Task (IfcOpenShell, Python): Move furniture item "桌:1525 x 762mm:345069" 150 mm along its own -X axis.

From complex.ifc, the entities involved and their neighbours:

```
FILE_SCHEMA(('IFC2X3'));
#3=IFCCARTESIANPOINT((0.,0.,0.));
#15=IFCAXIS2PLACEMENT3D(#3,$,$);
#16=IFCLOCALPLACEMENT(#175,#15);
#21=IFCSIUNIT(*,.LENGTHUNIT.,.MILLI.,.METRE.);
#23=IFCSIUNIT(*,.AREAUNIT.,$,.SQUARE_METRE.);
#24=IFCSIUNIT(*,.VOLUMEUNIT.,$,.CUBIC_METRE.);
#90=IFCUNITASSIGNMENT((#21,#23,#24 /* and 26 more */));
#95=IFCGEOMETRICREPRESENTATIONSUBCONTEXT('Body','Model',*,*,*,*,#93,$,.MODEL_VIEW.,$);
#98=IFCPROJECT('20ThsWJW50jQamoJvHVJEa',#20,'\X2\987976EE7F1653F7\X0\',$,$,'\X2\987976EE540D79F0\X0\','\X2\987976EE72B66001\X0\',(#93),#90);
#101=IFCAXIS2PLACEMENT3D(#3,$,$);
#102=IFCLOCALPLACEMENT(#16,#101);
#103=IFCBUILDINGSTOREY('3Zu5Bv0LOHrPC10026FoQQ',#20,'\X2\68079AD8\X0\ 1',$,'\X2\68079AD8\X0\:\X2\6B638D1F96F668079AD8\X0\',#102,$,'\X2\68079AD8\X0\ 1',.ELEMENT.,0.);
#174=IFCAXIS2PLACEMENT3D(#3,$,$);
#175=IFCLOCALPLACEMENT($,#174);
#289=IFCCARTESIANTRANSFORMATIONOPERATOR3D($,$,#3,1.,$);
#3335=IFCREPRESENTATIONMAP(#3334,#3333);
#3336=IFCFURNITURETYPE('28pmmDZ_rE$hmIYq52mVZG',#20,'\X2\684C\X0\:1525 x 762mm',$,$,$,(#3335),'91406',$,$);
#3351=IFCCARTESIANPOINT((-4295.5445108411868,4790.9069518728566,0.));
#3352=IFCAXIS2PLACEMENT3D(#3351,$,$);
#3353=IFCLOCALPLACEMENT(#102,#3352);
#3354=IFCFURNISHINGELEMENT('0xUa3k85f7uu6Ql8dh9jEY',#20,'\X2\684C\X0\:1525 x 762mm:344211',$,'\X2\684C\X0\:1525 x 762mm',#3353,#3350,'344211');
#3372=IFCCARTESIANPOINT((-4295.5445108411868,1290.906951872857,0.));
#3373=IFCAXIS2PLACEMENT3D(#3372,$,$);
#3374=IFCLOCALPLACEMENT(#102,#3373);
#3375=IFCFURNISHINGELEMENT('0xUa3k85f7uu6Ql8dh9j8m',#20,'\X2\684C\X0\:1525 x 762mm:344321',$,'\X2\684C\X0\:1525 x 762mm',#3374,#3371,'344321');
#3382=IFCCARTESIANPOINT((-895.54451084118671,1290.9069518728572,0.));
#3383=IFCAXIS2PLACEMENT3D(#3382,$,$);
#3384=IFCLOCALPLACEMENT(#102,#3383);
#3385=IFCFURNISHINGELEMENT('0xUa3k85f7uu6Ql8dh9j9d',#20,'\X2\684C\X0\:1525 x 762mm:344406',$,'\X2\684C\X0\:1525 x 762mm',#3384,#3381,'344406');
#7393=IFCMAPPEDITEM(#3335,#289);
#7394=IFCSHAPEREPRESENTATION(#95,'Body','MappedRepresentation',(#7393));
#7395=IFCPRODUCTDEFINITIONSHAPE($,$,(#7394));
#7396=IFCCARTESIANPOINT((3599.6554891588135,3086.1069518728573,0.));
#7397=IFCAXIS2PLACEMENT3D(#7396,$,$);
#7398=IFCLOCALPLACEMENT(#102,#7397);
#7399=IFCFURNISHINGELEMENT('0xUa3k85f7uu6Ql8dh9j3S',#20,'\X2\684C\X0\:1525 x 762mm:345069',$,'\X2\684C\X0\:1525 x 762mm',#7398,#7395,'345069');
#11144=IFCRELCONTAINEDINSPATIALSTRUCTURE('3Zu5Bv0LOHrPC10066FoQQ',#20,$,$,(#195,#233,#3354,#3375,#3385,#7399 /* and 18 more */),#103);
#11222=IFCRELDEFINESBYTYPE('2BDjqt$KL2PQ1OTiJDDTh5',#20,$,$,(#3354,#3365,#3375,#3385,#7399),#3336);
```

```python
import ifcopenshell
import ifcopenshell.api.geometry
import ifcopenshell.util.placement

model = ifcopenshell.open("complex.ifc")

item = model.by_guid("0xUa3k85f7uu6Ql8dh9j3S")
matrix = ifcopenshell.util.placement.get_local_placement(item.ObjectPlacement)
matrix[:3, 3] -= matrix[:3, 0] * 150.0
ifcopenshell.api.geometry.edit_object_placement(model, product=item, matrix=matrix, is_si=False)

print(ifcopenshell.util.placement.get_local_placement(item.ObjectPlacement).round(3) + 0.0)

model.write("complex_rev.ifc")
```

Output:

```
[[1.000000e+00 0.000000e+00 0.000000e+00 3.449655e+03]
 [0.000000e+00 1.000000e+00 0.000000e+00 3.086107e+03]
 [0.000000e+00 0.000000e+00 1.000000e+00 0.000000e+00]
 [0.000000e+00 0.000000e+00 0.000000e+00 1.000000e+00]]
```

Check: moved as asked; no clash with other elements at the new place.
